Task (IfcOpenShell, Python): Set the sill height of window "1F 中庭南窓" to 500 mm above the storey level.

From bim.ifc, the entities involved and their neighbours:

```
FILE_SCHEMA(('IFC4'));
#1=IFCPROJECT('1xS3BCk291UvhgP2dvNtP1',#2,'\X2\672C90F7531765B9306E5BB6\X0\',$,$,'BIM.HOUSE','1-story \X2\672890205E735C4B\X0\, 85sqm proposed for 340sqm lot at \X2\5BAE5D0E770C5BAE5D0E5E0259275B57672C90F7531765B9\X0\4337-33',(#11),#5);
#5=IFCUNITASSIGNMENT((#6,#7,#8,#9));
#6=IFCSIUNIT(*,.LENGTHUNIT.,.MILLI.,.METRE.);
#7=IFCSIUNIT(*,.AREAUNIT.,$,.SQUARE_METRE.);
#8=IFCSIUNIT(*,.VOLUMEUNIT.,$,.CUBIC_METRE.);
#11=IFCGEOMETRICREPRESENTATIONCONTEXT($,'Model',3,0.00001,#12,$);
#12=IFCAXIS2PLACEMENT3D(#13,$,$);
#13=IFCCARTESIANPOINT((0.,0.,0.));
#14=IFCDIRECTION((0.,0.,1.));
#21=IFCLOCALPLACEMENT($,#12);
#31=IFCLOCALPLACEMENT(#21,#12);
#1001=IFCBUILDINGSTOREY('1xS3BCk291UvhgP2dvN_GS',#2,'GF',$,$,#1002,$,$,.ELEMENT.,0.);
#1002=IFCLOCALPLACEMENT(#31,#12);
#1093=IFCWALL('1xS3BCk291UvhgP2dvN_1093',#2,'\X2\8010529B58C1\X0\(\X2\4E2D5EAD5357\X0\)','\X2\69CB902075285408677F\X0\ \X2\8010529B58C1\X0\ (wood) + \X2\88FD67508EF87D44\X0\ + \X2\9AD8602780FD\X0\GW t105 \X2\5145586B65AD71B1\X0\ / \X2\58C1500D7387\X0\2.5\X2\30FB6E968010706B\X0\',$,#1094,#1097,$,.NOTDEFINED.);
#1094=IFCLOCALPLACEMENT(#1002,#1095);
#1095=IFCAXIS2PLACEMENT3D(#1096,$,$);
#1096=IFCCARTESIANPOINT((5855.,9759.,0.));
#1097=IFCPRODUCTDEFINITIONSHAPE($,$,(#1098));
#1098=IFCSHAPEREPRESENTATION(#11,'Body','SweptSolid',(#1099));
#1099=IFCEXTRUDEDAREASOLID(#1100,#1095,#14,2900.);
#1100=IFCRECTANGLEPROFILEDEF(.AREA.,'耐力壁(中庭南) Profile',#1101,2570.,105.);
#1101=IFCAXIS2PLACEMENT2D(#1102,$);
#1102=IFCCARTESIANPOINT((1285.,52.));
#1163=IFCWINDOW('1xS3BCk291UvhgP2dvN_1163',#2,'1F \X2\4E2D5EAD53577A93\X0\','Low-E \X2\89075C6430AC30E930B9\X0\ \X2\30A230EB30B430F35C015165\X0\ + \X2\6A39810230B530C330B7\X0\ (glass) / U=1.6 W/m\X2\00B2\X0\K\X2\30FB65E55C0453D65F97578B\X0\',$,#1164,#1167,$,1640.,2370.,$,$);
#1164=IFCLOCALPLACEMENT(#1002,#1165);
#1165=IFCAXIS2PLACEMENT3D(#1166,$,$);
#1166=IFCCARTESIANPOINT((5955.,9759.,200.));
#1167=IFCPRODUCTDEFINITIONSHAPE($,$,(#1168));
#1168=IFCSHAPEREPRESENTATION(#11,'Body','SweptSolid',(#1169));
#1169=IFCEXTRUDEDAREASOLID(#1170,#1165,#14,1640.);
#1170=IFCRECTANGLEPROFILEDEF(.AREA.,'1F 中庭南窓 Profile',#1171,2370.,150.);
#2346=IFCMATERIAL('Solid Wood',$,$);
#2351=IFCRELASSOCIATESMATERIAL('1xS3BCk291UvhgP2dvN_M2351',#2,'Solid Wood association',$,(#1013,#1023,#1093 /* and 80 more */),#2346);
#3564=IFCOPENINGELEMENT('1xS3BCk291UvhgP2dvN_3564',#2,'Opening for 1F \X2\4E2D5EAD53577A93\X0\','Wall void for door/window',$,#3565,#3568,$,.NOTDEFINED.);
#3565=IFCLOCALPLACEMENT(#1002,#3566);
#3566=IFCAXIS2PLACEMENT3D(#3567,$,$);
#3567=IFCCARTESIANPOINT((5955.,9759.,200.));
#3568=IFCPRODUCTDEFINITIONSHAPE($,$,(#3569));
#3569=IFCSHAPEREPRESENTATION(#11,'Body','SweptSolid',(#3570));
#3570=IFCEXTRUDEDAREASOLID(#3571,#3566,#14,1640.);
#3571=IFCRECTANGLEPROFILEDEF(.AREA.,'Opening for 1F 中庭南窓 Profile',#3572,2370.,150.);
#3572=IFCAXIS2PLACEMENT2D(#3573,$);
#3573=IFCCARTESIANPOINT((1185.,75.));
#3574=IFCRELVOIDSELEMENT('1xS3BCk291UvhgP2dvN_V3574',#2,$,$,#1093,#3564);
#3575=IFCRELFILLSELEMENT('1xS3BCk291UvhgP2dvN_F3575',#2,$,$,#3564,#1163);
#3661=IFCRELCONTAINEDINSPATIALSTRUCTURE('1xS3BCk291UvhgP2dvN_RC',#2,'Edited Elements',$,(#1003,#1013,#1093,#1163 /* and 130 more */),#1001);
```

```python
import numpy as np
import ifcopenshell
import ifcopenshell.api.geometry
import ifcopenshell.geom
import ifcopenshell.util.element
import ifcopenshell.util.placement
import ifcopenshell.util.shape
import ifcopenshell.util.unit

model = ifcopenshell.open("bim.ifc")
unit_scale = ifcopenshell.util.unit.calculate_unit_scale(model)

window = model.by_id(1163)
opening = window.FillsVoids[0].RelatingOpeningElement
storey = ifcopenshell.util.element.get_container(window, ifc_class="IfcBuildingStorey")
level = ifcopenshell.util.placement.get_local_placement(storey.ObjectPlacement)[2, 3]

# The opening's origin need not be at the sill, so measure its lowest point.
shape = ifcopenshell.geom.create_shape(ifcopenshell.geom.settings(), opening)
bottom = ifcopenshell.util.shape.get_shape_bottom_elevation(shape, shape.geometry) / unit_scale
dz = level + 500.0 - bottom

shift = np.array([0.0, 0.0, dz])
# The window is not placed relative to its opening, so move both.
for product in (opening, window):
    matrix = ifcopenshell.util.placement.get_local_placement(product.ObjectPlacement)
    matrix[:3, 3] += shift
    ifcopenshell.api.geometry.edit_object_placement(model, product=product, matrix=matrix, is_si=False)

print(f"moved by {dz * unit_scale:+.3f} m")

model.write("bim-out.ifc")
```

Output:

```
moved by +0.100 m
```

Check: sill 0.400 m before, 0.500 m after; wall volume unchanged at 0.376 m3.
